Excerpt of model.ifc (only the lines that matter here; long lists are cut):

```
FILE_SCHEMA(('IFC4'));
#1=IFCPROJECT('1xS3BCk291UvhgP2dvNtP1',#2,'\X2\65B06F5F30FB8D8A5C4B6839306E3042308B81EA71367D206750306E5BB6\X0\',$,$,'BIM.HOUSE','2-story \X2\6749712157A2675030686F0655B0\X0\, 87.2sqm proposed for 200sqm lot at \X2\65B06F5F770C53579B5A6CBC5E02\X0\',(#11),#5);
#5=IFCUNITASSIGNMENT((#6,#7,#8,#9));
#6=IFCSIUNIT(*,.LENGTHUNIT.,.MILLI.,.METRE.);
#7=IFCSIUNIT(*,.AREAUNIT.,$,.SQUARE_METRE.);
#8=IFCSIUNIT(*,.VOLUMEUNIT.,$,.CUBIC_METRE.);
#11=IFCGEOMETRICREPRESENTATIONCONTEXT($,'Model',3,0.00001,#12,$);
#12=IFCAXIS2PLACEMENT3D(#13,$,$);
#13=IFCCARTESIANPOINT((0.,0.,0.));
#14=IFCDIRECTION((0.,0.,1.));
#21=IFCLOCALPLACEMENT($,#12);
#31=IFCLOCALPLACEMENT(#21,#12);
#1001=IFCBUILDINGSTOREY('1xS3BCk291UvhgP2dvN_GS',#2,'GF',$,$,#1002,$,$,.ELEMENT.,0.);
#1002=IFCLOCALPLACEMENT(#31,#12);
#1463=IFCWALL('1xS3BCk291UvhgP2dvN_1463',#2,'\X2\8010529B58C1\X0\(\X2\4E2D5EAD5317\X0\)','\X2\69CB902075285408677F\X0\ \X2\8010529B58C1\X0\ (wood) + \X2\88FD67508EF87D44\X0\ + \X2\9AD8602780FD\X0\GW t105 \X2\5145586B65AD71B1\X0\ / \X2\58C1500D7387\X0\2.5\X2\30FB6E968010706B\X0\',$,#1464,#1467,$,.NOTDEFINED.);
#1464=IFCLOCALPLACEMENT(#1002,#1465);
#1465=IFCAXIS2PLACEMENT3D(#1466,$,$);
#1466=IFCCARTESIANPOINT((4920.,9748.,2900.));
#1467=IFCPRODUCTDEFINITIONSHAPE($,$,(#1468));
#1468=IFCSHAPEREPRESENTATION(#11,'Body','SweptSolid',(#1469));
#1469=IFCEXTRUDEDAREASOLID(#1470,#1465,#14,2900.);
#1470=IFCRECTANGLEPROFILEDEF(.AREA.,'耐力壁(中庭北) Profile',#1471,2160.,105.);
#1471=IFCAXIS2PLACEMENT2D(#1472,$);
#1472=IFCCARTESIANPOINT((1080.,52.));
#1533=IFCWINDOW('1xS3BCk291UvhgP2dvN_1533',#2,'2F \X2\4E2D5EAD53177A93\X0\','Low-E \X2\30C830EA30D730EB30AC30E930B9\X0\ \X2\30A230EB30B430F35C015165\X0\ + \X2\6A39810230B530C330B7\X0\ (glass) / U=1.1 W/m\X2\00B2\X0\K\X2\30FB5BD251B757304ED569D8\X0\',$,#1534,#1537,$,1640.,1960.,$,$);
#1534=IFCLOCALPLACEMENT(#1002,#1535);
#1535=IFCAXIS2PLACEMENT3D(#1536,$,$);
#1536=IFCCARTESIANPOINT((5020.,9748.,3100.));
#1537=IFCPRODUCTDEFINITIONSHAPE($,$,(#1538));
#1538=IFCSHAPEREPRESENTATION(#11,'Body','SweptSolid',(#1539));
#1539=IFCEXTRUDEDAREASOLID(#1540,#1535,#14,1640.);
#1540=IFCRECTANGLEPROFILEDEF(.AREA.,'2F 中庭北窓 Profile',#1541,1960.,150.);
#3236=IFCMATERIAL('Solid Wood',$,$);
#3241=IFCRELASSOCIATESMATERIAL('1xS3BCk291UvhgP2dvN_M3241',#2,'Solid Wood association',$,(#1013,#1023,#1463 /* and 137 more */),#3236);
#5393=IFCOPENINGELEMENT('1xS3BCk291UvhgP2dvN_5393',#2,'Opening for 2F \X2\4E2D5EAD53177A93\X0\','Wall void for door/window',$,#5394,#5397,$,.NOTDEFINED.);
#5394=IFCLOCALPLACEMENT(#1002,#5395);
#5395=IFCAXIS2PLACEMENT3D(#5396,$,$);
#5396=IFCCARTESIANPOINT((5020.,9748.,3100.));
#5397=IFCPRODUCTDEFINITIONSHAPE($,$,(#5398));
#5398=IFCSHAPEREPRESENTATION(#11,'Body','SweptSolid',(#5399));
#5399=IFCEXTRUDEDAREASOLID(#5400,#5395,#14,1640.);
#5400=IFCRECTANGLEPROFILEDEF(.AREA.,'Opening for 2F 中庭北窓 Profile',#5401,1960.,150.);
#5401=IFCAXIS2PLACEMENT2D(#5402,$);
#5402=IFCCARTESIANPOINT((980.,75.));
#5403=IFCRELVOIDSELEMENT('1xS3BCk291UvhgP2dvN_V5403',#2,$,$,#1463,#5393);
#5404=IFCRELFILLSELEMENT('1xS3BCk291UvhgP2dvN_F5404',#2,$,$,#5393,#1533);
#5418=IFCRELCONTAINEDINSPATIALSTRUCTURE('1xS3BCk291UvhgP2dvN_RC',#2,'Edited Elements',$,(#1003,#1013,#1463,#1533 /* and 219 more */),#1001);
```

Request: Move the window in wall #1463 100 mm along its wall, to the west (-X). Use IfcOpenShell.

```python
import ifcopenshell
import ifcopenshell.api.geometry
import ifcopenshell.util.placement
import ifcopenshell.util.unit

model = ifcopenshell.open("model.ifc")
unit_scale = ifcopenshell.util.unit.calculate_unit_scale(model)

window = model.by_guid("1xS3BCk291UvhgP2dvN_1533")
opening = window.FillsVoids[0].RelatingOpeningElement
wall = opening.VoidsElements[0].RelatingBuildingElement

wall_matrix = ifcopenshell.util.placement.get_local_placement(wall.ObjectPlacement)
shift = wall_matrix[:3, 0] * -0.1 / unit_scale
before = ifcopenshell.util.placement.get_local_placement(window.ObjectPlacement)[:3, 3].copy()

# The window is not placed relative to its opening, so move both.
for product in (opening, window):
    matrix = ifcopenshell.util.placement.get_local_placement(product.ObjectPlacement)
    matrix[:3, 3] += shift
    ifcopenshell.api.geometry.edit_object_placement(model, product=product, matrix=matrix, is_si=False)

after = ifcopenshell.util.placement.get_local_placement(window.ObjectPlacement)[:3, 3]
print("window moved by", (after - before).round(3) + 0.0)

model.write("model_edited.ifc")
```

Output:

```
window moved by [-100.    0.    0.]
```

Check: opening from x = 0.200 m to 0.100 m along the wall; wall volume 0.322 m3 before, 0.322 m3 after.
